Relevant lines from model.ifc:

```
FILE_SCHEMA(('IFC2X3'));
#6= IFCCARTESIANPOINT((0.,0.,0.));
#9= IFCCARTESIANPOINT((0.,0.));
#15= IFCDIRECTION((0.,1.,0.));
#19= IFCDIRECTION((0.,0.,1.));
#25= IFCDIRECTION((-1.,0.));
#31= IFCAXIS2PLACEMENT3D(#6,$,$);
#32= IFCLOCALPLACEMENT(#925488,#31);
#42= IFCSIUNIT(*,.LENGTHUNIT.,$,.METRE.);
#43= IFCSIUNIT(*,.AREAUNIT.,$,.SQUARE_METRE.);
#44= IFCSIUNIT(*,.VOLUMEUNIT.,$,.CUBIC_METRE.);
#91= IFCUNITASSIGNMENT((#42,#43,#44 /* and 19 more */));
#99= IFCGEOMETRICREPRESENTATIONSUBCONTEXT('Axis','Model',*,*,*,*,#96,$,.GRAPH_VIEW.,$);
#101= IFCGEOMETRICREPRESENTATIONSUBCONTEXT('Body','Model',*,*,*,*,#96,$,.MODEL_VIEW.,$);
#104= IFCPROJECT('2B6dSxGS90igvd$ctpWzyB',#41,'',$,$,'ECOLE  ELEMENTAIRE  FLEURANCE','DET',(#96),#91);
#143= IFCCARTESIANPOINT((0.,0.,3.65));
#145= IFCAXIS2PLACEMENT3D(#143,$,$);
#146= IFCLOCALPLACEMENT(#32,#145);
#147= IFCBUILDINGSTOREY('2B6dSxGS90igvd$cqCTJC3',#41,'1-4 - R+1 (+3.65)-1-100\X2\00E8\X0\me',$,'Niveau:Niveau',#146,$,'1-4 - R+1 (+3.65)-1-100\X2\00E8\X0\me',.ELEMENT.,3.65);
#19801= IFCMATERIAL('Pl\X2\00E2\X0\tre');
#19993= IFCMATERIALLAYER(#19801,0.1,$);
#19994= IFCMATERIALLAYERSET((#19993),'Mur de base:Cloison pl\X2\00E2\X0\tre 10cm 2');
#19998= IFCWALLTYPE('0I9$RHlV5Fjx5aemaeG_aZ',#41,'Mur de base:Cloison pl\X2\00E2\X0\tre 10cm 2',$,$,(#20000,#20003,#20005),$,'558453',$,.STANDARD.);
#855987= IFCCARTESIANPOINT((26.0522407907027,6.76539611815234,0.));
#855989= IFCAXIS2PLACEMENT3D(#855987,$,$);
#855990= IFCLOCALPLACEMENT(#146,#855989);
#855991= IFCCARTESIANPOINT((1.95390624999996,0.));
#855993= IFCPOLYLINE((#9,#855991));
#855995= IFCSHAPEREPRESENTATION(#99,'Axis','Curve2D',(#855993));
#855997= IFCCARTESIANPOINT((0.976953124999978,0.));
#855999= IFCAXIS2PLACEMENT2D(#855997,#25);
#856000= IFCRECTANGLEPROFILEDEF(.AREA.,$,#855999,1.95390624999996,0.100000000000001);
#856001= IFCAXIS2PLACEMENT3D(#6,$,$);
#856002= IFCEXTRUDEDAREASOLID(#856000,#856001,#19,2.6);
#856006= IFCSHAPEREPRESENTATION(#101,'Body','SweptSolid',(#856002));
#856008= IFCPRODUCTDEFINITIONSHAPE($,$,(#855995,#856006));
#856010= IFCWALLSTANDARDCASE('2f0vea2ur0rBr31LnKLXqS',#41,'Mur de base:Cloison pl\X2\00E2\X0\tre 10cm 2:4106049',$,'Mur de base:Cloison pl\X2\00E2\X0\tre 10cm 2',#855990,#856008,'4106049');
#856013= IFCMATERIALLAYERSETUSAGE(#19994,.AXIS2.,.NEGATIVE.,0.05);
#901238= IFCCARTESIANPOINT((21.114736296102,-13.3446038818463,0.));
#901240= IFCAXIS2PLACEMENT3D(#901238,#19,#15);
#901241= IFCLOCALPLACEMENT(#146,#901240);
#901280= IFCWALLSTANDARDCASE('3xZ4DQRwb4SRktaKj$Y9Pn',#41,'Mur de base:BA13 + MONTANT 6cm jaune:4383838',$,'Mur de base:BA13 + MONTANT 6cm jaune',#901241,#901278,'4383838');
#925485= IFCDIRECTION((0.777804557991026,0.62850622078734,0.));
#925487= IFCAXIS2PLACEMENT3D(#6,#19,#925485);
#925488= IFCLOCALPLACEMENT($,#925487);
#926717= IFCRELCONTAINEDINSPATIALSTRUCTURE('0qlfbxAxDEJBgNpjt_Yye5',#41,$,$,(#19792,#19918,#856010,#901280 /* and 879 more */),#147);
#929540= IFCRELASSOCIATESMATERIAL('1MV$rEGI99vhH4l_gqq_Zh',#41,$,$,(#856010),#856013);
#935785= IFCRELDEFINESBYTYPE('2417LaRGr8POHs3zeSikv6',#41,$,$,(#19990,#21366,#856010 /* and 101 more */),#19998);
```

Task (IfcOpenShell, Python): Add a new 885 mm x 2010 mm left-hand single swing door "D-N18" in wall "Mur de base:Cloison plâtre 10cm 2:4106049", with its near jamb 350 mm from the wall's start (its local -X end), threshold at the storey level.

```python
import numpy as np
import ifcopenshell
import ifcopenshell.api.feature
import ifcopenshell.api.geometry
import ifcopenshell.api.root
import ifcopenshell.api.spatial
import ifcopenshell.api.type
import ifcopenshell.geom
import ifcopenshell.util.element
import ifcopenshell.util.placement
import ifcopenshell.util.representation
import ifcopenshell.util.shape
import ifcopenshell.util.unit

model = ifcopenshell.open("model.ifc")
unit_scale = ifcopenshell.util.unit.calculate_unit_scale(model)
settings = ifcopenshell.geom.settings()


def volume(element):
    """Net volume in cubic metres, openings subtracted."""
    shape = ifcopenshell.geom.create_shape(settings, element)
    return ifcopenshell.util.shape.get_volume(shape.geometry)


wall = model.by_guid("2f0vea2ur0rBr31LnKLXqS")
storey = ifcopenshell.util.element.get_container(wall, ifc_class="IfcBuildingStorey")
context = ifcopenshell.util.representation.get_context(model, "Model", "Body", "MODEL_VIEW")
before = volume(wall)

width, height, from_end, sill = 0.885, 2.01, 0.35, 0.0  # metres

# The wall runs along its own X axis, and the end named is its -X end.
wall_shape = ifcopenshell.geom.create_shape(settings, wall)
x, y, z = ifcopenshell.util.shape.get_vertices(wall_shape.geometry).T
start = x.min() + from_end
face, thickness = float(y.min()), float(y.max() - y.min())
wall_matrix = ifcopenshell.util.placement.get_local_placement(wall.ObjectPlacement)
level = ifcopenshell.util.placement.get_local_placement(storey.ObjectPlacement)[2, 3]


def in_wall(x, y):
    """Placement at x, y metres in the wall's axes, at sill height."""
    matrix = wall_matrix.copy()
    matrix[:, 3] = wall_matrix @ np.array([x / unit_scale, y / unit_scale, 0.0, 1.0])
    matrix[2, 3] = level + sill / unit_scale
    return matrix


# Opening: a box that overshoots both wall faces by 50 mm.
opening = ifcopenshell.api.root.create_entity(model, ifc_class="IfcOpeningElement")
box = ifcopenshell.api.geometry.add_wall_representation(
    model, context=context, length=width, height=height, thickness=thickness + 0.1
)
ifcopenshell.api.geometry.assign_representation(model, product=opening, representation=box)
ifcopenshell.api.geometry.edit_object_placement(model, product=opening, matrix=in_wall(start, face - 0.05), is_si=False)
ifcopenshell.api.feature.add_feature(model, feature=opening, element=wall)

door = ifcopenshell.api.root.create_entity(model, ifc_class="IfcDoor", name="D-N18")
door.OverallWidth, door.OverallHeight = width / unit_scale, height / unit_scale
body = ifcopenshell.api.geometry.add_door_representation(
    model,
    context=context,
    overall_width=door.OverallWidth,
    overall_height=door.OverallHeight,
    operation_type="SINGLE_SWING_LEFT",
    lining_properties={"LiningDepth": thickness / unit_scale, "ThresholdDepth": thickness / unit_scale},
)
ifcopenshell.api.geometry.assign_representation(model, product=door, representation=body)
ifcopenshell.api.spatial.assign_container(model, products=[door], relating_structure=storey)
fills = ifcopenshell.api.feature.add_filling(model, opening=opening, element=door)
fills.OwnerHistory = door.OwnerHistory  # required in IFC2X3

# IFC2X3 keeps the operation on the door style.
style = ifcopenshell.api.root.create_entity(model, ifc_class="IfcDoorStyle", name="D-N18")
style.OperationType, style.ConstructionType = "SINGLE_SWING_LEFT", "NOTDEFINED"
style.ParameterTakesPrecedence = style.Sizeable = False
ifcopenshell.api.type.assign_type(model, related_objects=[door], relating_type=style)

# The lining spans the wall, so the door starts at the wall face.
ifcopenshell.api.geometry.edit_object_placement(model, product=door, matrix=in_wall(start, face), is_si=False)

after = volume(wall)

print(f"wall volume {before:.3f} -> {after:.3f} m3")

model.write("model-out.ifc")
```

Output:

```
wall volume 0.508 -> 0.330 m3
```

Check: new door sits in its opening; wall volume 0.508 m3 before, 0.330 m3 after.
